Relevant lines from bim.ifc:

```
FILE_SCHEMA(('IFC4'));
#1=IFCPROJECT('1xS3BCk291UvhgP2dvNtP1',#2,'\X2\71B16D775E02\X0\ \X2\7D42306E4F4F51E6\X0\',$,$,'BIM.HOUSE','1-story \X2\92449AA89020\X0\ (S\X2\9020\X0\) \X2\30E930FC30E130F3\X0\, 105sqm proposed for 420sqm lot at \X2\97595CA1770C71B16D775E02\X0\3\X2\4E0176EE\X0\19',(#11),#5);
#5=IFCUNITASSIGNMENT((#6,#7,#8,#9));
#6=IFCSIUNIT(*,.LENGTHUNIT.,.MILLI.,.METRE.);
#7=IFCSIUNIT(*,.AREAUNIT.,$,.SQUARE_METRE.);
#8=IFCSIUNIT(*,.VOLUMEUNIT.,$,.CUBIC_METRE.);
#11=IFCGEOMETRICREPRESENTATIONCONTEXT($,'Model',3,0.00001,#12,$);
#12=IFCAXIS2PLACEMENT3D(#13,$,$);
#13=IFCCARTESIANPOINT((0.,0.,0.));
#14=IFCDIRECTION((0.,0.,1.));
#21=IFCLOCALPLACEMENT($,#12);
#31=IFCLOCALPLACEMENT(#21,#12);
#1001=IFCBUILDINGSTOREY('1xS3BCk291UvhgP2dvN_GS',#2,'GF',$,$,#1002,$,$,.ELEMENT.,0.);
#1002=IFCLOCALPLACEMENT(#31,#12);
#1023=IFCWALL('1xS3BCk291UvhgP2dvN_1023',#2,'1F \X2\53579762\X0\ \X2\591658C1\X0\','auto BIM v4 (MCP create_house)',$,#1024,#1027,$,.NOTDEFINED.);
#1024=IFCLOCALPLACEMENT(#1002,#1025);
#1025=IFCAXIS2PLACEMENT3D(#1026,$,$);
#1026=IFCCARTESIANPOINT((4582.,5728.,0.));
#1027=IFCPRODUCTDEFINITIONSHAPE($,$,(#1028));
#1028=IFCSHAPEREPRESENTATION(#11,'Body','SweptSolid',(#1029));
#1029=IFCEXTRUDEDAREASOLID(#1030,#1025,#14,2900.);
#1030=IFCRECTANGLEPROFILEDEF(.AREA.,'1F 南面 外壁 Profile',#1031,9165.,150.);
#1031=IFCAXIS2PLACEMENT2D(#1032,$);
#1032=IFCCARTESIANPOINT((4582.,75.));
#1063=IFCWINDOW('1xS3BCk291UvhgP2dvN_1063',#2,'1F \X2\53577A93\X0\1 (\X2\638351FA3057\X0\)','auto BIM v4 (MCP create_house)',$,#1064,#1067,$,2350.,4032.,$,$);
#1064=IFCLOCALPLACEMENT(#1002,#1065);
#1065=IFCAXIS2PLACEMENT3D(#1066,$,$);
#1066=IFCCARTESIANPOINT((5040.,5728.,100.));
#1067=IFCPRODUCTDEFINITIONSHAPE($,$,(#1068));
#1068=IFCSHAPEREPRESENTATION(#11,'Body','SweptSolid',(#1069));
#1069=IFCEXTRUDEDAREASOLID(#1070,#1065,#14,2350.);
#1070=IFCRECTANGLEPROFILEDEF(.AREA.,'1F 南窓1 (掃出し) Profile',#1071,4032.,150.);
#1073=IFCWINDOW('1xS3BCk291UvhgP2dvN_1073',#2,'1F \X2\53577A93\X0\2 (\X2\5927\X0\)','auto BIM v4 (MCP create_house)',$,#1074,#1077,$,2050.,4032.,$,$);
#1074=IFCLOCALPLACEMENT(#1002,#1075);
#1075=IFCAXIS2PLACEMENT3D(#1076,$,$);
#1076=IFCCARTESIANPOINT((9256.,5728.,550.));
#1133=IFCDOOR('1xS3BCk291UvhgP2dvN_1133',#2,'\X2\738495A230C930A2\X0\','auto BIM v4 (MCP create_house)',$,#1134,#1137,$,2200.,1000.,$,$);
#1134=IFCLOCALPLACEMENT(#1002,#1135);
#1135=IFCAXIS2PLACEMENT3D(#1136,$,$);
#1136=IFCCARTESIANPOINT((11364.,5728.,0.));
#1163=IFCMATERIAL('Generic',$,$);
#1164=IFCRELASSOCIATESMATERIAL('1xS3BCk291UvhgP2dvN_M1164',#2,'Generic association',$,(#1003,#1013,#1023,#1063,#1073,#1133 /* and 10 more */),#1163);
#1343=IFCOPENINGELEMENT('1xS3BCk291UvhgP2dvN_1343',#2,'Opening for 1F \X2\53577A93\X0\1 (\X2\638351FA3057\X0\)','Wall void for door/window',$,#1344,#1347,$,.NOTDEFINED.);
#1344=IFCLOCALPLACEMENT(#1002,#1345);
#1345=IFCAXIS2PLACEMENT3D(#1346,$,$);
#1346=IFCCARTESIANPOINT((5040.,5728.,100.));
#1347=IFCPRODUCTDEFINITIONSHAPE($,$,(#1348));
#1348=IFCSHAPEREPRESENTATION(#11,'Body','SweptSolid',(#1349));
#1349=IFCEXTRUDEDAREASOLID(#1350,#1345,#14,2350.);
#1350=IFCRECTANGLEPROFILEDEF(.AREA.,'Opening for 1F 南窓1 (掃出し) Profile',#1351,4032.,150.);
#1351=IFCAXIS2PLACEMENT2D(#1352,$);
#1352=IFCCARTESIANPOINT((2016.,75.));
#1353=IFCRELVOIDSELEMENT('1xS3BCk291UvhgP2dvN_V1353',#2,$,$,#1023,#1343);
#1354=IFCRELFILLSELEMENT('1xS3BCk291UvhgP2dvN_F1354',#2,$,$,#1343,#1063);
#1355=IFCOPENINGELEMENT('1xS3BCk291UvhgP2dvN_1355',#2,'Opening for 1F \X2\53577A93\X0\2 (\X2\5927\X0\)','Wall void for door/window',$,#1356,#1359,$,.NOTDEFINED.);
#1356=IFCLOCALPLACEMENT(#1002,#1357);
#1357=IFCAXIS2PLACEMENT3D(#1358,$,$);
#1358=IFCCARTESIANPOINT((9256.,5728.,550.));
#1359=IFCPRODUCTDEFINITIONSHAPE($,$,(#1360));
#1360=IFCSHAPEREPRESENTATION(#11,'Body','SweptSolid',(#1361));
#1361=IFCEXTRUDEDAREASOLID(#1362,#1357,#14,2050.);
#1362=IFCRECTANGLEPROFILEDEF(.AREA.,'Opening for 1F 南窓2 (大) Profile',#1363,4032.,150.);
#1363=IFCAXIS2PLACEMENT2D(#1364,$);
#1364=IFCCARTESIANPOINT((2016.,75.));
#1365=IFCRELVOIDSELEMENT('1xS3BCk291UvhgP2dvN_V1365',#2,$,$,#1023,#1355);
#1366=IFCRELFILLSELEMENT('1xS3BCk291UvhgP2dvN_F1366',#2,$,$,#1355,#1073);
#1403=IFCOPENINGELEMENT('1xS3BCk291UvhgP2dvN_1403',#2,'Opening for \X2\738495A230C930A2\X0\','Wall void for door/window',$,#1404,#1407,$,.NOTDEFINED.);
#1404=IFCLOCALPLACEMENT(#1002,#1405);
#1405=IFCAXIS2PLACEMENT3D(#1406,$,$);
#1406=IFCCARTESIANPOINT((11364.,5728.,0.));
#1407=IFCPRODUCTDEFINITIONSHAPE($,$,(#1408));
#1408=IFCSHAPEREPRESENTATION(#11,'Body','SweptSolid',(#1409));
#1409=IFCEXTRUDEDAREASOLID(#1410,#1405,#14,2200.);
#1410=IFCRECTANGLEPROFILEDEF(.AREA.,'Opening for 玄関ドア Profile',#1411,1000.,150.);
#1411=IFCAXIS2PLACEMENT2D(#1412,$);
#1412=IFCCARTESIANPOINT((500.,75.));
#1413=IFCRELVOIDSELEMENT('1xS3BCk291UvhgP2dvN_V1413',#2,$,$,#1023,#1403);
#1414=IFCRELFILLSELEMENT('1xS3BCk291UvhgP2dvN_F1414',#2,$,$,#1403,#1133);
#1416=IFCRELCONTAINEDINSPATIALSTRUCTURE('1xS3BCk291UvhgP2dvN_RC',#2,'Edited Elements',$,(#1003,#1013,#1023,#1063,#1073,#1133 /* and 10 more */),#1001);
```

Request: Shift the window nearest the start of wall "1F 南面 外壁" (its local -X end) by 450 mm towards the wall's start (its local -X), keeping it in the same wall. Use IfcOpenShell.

```python
import ifcopenshell
import ifcopenshell.api.geometry
import ifcopenshell.util.placement

model = ifcopenshell.open("bim.ifc")

window = model.by_guid("1xS3BCk291UvhgP2dvN_1063")
opening = window.FillsVoids[0].RelatingOpeningElement
wall = opening.VoidsElements[0].RelatingBuildingElement

wall_matrix = ifcopenshell.util.placement.get_local_placement(wall.ObjectPlacement)
shift = wall_matrix[:3, 0] * -450.0
before = ifcopenshell.util.placement.get_local_placement(window.ObjectPlacement)[:3, 3].copy()

# The window is not placed relative to its opening, so move both.
for product in (opening, window):
    matrix = ifcopenshell.util.placement.get_local_placement(product.ObjectPlacement)
    matrix[:3, 3] += shift
    ifcopenshell.api.geometry.edit_object_placement(model, product=product, matrix=matrix, is_si=False)

after = ifcopenshell.util.placement.get_local_placement(window.ObjectPlacement)[:3, 3]
print("window moved by", (after - before).round(3) + 0.0)

model.write("bim_updated.ifc")
```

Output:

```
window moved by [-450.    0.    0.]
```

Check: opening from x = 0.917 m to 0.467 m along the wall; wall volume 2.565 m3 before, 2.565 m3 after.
